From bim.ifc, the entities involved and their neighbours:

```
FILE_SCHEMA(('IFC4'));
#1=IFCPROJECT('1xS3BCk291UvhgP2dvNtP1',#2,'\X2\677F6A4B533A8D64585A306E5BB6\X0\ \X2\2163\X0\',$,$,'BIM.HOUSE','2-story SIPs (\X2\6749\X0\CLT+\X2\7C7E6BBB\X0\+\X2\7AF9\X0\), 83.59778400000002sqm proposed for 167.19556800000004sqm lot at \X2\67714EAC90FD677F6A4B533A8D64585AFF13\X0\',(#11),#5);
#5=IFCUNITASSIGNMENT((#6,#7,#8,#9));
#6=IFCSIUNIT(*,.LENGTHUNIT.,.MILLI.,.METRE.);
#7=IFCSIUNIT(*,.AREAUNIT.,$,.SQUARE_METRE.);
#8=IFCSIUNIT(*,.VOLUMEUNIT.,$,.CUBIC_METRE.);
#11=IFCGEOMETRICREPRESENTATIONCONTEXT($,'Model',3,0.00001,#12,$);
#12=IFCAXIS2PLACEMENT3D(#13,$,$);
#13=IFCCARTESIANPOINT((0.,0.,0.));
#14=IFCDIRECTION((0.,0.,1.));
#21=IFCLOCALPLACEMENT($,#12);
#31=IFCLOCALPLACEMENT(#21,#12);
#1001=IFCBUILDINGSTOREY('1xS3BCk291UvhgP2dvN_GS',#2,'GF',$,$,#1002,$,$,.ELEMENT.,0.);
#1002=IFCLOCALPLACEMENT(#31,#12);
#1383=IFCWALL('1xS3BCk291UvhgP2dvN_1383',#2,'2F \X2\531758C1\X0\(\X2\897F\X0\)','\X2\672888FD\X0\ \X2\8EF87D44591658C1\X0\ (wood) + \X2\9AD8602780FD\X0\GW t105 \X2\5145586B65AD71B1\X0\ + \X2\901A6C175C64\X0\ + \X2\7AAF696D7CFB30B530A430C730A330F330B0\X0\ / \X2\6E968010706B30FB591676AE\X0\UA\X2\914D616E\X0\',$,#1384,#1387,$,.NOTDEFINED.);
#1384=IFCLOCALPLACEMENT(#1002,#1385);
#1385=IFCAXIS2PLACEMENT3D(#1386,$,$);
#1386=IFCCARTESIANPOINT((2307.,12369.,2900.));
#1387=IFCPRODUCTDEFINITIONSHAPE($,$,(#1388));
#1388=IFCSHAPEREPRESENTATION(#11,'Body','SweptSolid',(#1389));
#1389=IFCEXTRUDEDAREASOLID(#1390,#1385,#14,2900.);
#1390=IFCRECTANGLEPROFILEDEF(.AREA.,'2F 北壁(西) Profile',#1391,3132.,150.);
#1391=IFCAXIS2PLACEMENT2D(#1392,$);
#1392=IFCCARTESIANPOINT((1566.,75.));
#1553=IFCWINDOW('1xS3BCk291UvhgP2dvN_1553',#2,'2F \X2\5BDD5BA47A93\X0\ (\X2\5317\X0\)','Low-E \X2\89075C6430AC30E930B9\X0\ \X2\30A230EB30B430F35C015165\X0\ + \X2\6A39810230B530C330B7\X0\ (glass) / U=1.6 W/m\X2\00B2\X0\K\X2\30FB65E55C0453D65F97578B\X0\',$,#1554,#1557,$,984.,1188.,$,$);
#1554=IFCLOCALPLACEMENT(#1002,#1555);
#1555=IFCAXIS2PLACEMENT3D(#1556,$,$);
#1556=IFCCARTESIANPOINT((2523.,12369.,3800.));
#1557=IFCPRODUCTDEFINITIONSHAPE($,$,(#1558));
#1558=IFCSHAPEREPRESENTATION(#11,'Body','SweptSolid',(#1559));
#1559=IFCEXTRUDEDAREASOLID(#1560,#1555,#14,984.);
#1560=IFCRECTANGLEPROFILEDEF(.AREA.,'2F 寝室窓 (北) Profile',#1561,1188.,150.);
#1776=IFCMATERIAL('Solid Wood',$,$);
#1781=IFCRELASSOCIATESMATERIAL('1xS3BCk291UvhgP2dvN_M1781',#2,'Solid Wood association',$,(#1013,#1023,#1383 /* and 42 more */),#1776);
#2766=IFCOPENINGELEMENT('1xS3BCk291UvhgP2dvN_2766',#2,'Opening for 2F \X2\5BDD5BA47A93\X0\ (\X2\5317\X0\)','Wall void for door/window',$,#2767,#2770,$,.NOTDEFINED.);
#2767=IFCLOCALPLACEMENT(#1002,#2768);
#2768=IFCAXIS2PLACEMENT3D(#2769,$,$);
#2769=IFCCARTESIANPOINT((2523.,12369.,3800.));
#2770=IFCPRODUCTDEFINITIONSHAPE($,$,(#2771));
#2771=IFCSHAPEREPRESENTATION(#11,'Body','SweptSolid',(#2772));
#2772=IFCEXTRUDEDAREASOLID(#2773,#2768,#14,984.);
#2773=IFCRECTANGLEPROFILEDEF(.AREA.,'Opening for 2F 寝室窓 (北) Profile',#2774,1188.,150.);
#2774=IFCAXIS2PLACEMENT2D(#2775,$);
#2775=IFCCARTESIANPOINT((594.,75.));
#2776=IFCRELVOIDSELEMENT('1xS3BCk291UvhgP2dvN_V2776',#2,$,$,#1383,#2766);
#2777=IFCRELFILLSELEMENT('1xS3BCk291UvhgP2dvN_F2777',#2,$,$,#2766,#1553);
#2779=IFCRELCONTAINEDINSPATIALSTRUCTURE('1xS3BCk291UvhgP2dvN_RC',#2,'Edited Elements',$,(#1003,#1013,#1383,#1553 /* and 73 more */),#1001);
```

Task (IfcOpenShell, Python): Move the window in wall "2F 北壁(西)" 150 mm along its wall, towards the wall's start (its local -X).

```python
import ifcopenshell
import ifcopenshell.api.geometry
import ifcopenshell.util.placement

model = ifcopenshell.open("bim.ifc")

window = model.by_id(1553)
opening = window.FillsVoids[0].RelatingOpeningElement
wall = opening.VoidsElements[0].RelatingBuildingElement

wall_matrix = ifcopenshell.util.placement.get_local_placement(wall.ObjectPlacement)
shift = wall_matrix[:3, 0] * -150.0
before = ifcopenshell.util.placement.get_local_placement(window.ObjectPlacement)[:3, 3].copy()

# The window is not placed relative to its opening, so move both.
for product in (opening, window):
    matrix = ifcopenshell.util.placement.get_local_placement(product.ObjectPlacement)
    matrix[:3, 3] += shift
    ifcopenshell.api.geometry.edit_object_placement(model, product=product, matrix=matrix, is_si=False)

after = ifcopenshell.util.placement.get_local_placement(window.ObjectPlacement)[:3, 3]
print("window moved by", (after - before).round(3) + 0.0)

model.write("bim_v2.ifc")
```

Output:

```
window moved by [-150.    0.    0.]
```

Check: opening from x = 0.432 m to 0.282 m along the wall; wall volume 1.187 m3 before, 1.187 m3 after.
